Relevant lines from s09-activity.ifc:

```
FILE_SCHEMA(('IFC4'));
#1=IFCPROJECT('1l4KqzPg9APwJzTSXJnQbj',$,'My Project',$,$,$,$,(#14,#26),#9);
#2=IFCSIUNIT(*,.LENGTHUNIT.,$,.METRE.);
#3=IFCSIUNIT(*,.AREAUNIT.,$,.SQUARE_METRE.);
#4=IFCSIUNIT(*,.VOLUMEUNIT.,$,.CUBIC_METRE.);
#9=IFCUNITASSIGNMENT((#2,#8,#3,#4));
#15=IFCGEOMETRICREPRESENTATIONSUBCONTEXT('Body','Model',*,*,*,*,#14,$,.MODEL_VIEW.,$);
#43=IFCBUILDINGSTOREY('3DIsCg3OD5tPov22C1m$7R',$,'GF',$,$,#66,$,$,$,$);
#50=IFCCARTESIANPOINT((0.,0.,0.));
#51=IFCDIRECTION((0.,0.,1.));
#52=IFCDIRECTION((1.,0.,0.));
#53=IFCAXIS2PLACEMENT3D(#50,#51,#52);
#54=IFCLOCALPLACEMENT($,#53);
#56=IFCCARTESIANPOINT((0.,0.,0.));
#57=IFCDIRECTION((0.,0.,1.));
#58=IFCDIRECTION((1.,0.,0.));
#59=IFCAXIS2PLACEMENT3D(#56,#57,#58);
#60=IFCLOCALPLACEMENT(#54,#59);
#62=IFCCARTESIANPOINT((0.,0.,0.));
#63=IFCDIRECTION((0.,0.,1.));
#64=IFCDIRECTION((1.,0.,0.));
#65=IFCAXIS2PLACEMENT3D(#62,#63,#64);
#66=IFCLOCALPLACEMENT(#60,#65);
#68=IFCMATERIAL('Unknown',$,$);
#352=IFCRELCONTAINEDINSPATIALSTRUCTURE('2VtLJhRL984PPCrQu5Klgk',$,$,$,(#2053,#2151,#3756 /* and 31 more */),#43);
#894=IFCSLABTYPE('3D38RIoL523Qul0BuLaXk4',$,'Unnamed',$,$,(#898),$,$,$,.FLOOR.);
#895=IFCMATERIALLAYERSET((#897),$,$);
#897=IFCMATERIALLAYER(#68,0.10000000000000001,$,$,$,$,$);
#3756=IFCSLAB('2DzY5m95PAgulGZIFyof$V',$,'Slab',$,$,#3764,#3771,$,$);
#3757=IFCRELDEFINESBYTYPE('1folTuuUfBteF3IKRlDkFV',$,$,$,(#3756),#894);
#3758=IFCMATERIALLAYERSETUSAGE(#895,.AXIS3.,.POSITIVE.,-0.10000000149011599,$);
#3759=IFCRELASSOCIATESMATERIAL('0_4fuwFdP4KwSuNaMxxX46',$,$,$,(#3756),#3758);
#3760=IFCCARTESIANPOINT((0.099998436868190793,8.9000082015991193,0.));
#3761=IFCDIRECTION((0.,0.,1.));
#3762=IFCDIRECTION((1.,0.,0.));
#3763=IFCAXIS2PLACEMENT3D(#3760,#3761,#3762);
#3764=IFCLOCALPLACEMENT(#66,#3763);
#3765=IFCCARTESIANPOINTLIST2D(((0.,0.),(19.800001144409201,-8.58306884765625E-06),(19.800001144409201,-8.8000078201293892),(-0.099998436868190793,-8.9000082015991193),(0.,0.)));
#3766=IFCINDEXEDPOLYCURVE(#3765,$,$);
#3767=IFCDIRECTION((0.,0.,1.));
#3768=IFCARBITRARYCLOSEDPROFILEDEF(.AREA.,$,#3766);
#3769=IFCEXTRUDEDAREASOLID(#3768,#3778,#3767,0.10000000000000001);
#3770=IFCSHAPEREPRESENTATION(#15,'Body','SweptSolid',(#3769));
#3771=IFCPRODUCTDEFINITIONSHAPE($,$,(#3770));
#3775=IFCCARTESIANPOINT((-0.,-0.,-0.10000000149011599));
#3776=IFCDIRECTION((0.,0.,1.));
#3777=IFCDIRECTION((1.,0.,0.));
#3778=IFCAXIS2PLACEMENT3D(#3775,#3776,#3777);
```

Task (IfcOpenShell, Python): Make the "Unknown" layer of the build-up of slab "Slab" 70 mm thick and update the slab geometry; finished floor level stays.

```python
import ifcopenshell
import ifcopenshell.util.element
import ifcopenshell.util.representation
import ifcopenshell.util.unit

model = ifcopenshell.open("s09-activity.ifc")
unit_scale = ifcopenshell.util.unit.calculate_unit_scale(model)

layer_set = model.by_id(895)
layer = next(l for l in layer_set.MaterialLayers if l.Material and l.Material.Name == "Unknown")
change = 0.07 / unit_scale - layer.LayerThickness
layer.LayerThickness += change

# Geometry does not follow the layer set by itself.
slabs = [e for e in ifcopenshell.util.element.get_elements_by_material(model, layer_set) if e.is_a("IfcSlab")]
for slab in sorted(slabs, key=lambda e: e.id()):
    body = ifcopenshell.util.representation.get_representation(slab, "Model", "Body")
    solid = body.Items[0]
    old_depth = solid.Depth
    solid.Depth += change
    # Extruded upwards: lower the start of the extrusion so the top stays.
    x, y, z = solid.Position.Location.Coordinates
    solid.Position.Location = model.createIfcCartesianPoint((x, y, z - change))
    print(slab.id(), f"{old_depth:g} -> {solid.Depth:g}")

# The layers are counted up from the underside, which has moved.
for usage in {ifcopenshell.util.element.get_material(slab) for slab in slabs}:
    usage.OffsetFromReferenceLine -= change

model.write("s09-activity_edited.ifc")
```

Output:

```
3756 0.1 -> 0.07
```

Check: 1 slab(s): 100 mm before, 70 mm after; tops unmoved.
